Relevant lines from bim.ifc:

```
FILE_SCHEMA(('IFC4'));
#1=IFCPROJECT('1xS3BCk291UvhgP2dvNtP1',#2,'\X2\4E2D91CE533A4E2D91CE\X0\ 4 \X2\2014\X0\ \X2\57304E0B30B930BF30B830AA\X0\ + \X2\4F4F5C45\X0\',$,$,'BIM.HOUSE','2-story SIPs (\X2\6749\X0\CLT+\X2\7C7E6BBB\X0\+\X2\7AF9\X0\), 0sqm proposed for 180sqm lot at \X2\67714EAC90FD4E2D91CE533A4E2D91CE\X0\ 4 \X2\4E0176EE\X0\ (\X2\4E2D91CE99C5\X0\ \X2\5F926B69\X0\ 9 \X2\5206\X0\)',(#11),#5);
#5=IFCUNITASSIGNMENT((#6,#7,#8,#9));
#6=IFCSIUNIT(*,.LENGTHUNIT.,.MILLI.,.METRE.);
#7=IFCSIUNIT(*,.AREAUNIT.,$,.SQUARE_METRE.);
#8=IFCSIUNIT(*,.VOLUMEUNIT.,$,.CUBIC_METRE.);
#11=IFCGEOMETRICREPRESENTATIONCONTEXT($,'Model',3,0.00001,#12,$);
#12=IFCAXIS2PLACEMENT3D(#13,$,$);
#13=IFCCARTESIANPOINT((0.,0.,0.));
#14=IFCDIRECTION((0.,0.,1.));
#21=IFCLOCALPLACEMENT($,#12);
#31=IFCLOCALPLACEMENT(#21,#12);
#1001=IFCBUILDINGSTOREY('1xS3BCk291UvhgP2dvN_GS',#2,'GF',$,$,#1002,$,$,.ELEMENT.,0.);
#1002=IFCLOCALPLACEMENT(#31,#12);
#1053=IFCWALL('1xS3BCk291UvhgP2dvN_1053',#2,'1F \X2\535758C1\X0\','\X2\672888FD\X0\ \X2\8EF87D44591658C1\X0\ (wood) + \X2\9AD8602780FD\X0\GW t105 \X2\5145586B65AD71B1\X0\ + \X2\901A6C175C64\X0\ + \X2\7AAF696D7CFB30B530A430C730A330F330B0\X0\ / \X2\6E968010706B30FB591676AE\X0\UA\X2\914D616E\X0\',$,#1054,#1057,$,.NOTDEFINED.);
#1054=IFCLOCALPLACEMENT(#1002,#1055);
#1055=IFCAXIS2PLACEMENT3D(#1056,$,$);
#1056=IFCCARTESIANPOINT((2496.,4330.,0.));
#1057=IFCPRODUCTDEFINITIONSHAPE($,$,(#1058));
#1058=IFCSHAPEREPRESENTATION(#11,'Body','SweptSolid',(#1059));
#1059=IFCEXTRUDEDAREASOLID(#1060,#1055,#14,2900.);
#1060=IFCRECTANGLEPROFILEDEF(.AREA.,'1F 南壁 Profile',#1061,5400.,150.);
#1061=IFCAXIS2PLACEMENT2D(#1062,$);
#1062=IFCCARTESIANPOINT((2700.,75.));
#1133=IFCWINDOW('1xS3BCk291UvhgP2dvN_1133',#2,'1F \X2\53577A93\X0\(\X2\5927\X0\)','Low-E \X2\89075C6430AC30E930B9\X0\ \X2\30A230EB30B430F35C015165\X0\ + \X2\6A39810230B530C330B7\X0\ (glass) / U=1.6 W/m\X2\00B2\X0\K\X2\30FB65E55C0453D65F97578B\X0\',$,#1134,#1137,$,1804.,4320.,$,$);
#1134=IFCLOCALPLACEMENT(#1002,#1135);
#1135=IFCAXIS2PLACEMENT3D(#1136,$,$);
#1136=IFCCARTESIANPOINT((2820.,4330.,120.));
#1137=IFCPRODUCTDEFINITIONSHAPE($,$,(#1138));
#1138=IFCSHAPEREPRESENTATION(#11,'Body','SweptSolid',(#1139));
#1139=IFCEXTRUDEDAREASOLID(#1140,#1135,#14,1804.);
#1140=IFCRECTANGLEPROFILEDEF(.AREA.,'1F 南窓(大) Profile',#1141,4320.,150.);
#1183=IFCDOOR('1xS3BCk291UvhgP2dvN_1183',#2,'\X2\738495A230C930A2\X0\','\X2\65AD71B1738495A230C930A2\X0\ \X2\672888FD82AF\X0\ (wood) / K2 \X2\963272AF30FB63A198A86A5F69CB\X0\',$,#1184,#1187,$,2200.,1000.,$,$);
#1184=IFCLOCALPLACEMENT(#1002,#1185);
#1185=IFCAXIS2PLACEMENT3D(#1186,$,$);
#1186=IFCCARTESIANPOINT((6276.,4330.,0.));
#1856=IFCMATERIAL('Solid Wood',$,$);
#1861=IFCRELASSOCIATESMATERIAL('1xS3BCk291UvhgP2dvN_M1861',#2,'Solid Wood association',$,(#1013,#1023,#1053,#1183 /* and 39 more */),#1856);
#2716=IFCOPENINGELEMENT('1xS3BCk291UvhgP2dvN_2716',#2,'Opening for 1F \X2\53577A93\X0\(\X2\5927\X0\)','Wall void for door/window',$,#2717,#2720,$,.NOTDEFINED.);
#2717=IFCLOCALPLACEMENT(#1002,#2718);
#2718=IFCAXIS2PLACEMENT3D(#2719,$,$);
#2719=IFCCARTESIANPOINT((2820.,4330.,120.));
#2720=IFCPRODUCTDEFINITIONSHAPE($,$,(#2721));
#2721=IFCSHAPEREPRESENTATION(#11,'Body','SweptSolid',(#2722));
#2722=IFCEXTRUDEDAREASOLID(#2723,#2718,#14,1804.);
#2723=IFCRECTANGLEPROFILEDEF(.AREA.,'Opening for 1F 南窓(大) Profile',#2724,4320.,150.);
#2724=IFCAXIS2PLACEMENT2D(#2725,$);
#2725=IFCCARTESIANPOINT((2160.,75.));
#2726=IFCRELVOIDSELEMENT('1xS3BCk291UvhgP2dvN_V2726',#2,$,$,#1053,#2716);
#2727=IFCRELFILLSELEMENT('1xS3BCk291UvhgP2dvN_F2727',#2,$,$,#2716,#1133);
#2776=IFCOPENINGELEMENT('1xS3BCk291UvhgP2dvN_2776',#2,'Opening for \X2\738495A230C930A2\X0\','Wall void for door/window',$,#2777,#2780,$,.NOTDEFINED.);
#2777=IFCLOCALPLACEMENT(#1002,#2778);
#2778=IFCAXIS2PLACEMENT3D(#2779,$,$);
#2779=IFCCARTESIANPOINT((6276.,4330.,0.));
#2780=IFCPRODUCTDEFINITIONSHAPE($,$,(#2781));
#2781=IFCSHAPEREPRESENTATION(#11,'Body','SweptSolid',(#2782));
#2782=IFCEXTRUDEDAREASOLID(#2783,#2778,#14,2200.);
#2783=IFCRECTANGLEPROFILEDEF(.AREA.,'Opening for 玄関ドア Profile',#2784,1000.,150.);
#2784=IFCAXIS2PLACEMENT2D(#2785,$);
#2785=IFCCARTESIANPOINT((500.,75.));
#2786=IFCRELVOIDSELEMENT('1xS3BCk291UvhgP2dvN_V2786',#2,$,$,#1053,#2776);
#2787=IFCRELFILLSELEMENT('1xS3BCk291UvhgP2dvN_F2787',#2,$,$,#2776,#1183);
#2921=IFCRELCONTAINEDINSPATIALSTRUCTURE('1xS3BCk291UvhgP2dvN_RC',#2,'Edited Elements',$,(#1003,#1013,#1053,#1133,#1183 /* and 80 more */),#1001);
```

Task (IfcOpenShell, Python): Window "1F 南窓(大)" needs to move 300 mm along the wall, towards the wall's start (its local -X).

```python
import ifcopenshell
import ifcopenshell.api.geometry
import ifcopenshell.util.placement

model = ifcopenshell.open("bim.ifc")

window = model.by_id(1133)
opening = window.FillsVoids[0].RelatingOpeningElement
wall = opening.VoidsElements[0].RelatingBuildingElement

wall_matrix = ifcopenshell.util.placement.get_local_placement(wall.ObjectPlacement)
shift = wall_matrix[:3, 0] * -300.0
before = ifcopenshell.util.placement.get_local_placement(window.ObjectPlacement)[:3, 3].copy()

# The window is not placed relative to its opening, so move both.
for product in (opening, window):
    matrix = ifcopenshell.util.placement.get_local_placement(product.ObjectPlacement)
    matrix[:3, 3] += shift
    ifcopenshell.api.geometry.edit_object_placement(model, product=product, matrix=matrix, is_si=False)

after = ifcopenshell.util.placement.get_local_placement(window.ObjectPlacement)[:3, 3]
print("window moved by", (after - before).round(3) + 0.0)

model.write("bim_updated.ifc")
```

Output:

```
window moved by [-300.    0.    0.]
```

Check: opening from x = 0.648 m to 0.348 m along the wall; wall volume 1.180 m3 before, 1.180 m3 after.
